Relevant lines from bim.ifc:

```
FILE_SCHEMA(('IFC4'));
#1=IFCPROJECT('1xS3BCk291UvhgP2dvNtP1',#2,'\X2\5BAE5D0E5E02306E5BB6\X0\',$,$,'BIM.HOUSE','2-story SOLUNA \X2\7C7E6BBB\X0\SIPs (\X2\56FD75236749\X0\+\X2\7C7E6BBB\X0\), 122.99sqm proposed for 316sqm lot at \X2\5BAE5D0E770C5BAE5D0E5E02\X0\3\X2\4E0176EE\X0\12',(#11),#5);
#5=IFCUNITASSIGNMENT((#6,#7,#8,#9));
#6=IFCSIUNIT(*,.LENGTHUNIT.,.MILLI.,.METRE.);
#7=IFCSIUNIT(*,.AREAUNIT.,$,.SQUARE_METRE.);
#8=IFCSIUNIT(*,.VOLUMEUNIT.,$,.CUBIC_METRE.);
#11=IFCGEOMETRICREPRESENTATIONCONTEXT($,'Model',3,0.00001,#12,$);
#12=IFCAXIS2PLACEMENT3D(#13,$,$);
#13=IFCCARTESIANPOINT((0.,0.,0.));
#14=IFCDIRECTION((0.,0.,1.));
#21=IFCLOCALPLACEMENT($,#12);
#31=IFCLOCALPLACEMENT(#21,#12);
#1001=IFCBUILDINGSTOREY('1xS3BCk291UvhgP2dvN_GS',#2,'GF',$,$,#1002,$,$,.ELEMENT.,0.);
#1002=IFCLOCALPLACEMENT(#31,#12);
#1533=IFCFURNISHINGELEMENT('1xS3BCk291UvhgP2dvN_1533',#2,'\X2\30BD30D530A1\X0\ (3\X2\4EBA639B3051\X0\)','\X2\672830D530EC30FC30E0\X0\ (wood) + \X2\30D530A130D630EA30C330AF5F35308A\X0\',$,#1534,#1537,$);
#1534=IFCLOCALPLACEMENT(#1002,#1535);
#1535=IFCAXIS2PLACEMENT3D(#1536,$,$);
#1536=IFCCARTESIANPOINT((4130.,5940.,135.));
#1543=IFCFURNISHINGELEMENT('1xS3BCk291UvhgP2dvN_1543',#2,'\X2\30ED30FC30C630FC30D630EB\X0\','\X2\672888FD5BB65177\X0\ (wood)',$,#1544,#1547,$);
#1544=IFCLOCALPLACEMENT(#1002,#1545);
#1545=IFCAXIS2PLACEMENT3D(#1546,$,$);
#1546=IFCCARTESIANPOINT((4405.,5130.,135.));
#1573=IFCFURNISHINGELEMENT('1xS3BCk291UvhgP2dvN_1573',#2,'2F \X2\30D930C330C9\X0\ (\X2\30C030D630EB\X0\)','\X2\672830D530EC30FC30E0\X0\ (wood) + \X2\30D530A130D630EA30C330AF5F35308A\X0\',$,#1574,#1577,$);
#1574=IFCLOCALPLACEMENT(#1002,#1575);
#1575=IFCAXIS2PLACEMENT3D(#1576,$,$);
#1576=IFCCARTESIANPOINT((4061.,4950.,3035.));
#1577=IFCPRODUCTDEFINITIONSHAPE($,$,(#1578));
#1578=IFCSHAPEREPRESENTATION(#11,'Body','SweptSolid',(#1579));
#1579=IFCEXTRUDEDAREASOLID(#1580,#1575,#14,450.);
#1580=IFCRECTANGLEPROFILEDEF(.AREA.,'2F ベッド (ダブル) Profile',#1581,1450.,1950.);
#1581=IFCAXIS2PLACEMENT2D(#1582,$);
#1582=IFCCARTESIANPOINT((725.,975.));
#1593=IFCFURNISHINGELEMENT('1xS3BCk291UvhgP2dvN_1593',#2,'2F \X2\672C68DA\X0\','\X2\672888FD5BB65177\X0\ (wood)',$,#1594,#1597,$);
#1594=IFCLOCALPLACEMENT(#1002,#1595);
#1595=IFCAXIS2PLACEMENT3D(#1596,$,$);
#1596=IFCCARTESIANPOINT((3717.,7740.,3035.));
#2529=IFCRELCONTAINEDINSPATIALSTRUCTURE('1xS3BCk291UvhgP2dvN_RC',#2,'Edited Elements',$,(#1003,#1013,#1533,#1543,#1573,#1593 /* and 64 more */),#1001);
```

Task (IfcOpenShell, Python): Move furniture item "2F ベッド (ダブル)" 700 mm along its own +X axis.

```python
import ifcopenshell
import ifcopenshell.api.geometry
import ifcopenshell.util.placement

model = ifcopenshell.open("bim.ifc")

item = model.by_guid("1xS3BCk291UvhgP2dvN_1573")
matrix = ifcopenshell.util.placement.get_local_placement(item.ObjectPlacement)
matrix[:3, 3] += matrix[:3, 0] * 700.0
ifcopenshell.api.geometry.edit_object_placement(model, product=item, matrix=matrix, is_si=False)

print(ifcopenshell.util.placement.get_local_placement(item.ObjectPlacement).round(3) + 0.0)

model.write("bim_updated.ifc")
```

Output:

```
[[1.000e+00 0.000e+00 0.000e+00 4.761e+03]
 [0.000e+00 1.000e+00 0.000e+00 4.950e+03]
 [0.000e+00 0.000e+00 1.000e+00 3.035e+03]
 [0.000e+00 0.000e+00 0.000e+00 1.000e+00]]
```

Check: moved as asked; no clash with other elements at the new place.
